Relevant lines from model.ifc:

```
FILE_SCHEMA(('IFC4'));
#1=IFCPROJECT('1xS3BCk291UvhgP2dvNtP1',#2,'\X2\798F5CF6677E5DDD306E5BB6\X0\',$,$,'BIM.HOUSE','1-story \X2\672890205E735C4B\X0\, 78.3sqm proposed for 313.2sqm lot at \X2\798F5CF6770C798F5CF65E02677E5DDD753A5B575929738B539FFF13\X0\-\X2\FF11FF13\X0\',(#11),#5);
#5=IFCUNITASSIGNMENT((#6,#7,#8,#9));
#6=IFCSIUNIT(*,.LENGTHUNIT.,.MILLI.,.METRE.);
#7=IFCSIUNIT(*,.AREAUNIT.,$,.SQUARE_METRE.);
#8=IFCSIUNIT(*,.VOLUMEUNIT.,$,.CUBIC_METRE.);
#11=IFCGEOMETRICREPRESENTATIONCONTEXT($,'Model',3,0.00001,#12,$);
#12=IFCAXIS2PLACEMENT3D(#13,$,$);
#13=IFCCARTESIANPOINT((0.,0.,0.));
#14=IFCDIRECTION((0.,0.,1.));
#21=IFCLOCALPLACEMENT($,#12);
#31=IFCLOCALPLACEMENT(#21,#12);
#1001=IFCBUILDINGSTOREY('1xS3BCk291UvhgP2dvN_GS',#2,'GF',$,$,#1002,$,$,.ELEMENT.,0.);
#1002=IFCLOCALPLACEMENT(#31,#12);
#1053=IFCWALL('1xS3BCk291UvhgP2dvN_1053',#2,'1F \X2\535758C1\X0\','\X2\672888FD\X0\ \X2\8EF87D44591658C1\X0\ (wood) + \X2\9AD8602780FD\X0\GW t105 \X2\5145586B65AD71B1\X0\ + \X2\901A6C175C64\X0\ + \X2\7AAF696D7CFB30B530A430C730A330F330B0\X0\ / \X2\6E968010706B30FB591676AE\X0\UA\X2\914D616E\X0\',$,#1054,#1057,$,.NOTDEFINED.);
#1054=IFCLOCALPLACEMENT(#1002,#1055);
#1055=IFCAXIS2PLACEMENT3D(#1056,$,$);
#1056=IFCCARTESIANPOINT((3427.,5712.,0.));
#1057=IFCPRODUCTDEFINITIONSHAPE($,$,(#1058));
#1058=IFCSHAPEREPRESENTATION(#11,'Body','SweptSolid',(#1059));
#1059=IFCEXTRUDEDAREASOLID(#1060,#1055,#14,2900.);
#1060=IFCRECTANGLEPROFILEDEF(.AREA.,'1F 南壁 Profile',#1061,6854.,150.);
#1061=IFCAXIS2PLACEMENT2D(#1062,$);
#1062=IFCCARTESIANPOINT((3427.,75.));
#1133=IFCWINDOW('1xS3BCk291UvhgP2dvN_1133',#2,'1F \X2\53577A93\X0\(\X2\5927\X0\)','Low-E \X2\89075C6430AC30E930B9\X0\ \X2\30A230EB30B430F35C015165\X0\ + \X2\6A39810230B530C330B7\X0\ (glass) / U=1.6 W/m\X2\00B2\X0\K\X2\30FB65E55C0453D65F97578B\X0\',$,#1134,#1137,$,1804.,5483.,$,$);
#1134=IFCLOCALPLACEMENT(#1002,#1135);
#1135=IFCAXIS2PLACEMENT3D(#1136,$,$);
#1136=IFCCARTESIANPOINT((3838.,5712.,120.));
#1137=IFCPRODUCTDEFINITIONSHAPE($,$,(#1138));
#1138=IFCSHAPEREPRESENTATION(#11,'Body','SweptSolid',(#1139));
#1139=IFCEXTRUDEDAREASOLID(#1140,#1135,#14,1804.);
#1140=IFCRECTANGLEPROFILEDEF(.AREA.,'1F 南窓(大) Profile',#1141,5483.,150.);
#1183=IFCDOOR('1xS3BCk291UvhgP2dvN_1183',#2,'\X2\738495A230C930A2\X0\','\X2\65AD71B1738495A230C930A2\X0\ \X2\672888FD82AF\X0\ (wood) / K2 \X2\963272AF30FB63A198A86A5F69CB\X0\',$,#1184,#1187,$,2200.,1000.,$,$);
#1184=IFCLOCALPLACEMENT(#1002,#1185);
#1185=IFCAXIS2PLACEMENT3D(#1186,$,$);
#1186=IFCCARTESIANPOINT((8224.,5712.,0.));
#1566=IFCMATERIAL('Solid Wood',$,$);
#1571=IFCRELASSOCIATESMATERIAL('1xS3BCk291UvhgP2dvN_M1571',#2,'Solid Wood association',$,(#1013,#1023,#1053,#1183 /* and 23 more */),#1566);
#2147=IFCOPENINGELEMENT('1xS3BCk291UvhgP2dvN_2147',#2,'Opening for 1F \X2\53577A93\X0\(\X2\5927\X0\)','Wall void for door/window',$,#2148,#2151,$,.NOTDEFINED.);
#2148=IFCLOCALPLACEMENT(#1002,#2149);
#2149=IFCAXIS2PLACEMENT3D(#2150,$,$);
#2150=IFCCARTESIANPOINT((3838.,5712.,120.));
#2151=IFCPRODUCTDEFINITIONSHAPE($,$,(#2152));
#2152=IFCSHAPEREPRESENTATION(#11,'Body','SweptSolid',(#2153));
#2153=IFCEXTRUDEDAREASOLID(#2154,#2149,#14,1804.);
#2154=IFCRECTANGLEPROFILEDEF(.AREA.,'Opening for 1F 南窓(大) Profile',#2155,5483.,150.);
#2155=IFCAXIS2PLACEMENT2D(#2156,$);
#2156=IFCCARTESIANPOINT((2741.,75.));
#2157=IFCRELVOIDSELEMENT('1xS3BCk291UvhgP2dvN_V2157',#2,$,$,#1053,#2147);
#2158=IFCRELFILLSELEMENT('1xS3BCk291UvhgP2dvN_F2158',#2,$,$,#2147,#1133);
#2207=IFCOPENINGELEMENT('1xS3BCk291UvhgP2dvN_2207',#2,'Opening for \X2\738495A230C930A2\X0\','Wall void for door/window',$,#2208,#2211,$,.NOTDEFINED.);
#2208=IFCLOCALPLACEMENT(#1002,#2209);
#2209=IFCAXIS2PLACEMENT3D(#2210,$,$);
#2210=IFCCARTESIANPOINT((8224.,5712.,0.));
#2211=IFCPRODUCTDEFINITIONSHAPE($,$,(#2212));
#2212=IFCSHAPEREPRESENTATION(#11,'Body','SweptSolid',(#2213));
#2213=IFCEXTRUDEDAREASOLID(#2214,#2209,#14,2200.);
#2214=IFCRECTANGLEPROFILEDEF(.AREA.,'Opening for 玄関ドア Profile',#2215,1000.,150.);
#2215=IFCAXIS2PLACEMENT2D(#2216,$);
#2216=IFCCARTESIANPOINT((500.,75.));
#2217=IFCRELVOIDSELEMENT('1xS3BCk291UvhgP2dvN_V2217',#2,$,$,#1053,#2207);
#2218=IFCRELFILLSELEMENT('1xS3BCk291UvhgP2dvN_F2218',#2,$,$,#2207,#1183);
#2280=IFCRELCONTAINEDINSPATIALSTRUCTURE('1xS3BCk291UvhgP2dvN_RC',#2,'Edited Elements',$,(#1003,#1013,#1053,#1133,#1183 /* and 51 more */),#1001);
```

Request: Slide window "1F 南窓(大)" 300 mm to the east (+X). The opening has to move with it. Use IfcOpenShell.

```python
import ifcopenshell
import ifcopenshell.api.geometry
import ifcopenshell.util.placement
import ifcopenshell.util.unit

model = ifcopenshell.open("model.ifc")
unit_scale = ifcopenshell.util.unit.calculate_unit_scale(model)

window = model.by_id(1133)
opening = window.FillsVoids[0].RelatingOpeningElement
wall = opening.VoidsElements[0].RelatingBuildingElement

wall_matrix = ifcopenshell.util.placement.get_local_placement(wall.ObjectPlacement)
shift = wall_matrix[:3, 0] * 0.3 / unit_scale
before = ifcopenshell.util.placement.get_local_placement(window.ObjectPlacement)[:3, 3].copy()

# The window is not placed relative to its opening, so move both.
for product in (opening, window):
    matrix = ifcopenshell.util.placement.get_local_placement(product.ObjectPlacement)
    matrix[:3, 3] += shift
    ifcopenshell.api.geometry.edit_object_placement(model, product=product, matrix=matrix, is_si=False)

after = ifcopenshell.util.placement.get_local_placement(window.ObjectPlacement)[:3, 3]
print("window moved by", (after - before).round(3) + 0.0)

model.write("model_rev.ifc")
```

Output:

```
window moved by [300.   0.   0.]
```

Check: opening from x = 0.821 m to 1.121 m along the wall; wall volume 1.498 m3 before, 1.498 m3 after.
